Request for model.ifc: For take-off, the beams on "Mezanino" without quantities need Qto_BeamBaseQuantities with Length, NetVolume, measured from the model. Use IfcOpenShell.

First a look at what the model holds.

```python
import ifcopenshell
import ifcopenshell.util.element
import ifcopenshell.util.unit

model = ifcopenshell.open("model.ifc")
print(model.schema)
for unit_type in ("LENGTHUNIT", "AREAUNIT", "VOLUMEUNIT"):
    print(unit_type, ifcopenshell.util.unit.calculate_unit_scale(model, unit_type))
storey = next(s for s in model.by_type("IfcBuildingStorey") if s.Name == "Mezanino")
beams = [e for e in ifcopenshell.util.element.get_decomposition(storey) if e.is_a("IfcBeam")]
for e in sorted(beams, key=lambda e: e.id()):
    print(e.id(), e.is_a(), e.Name, list(ifcopenshell.util.element.get_psets(e, qtos_only=True)), sep=" | ")
```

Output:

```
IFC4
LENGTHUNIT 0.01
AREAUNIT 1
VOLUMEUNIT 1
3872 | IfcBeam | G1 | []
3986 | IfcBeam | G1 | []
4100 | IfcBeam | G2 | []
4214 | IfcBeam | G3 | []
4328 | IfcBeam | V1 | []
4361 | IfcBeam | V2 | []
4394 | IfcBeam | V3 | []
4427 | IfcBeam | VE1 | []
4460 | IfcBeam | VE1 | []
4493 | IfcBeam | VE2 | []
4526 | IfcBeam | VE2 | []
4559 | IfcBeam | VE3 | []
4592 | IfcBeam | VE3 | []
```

```python
import ifcopenshell
import ifcopenshell.api.pset
import ifcopenshell.geom
import ifcopenshell.util.element
import ifcopenshell.util.shape
import ifcopenshell.util.unit

model = ifcopenshell.open("model.ifc")
unit_scale = ifcopenshell.util.unit.calculate_unit_scale(model)
volume_scale = ifcopenshell.util.unit.calculate_unit_scale(model, "VOLUMEUNIT")
settings = ifcopenshell.geom.settings()

storey = next(s for s in model.by_type("IfcBuildingStorey") if s.Name == "Mezanino")
beams = [e for e in ifcopenshell.util.element.get_decomposition(storey) if e.is_a("IfcBeam")]

for e in sorted(beams, key=lambda e: e.id()):
    if ifcopenshell.util.element.get_psets(e, qtos_only=True, should_inherit=False):
        continue
    # Geometry comes back in metres, in the element's own axes.
    shape = ifcopenshell.geom.create_shape(settings, e)
    values = {
        "Length": ifcopenshell.util.shape.get_max_xyz(shape.geometry) / unit_scale,
        "NetVolume": ifcopenshell.util.shape.get_volume(shape.geometry) / volume_scale,
    }
    qto = ifcopenshell.api.pset.add_qto(model, product=e, name="Qto_BeamBaseQuantities")
    ifcopenshell.api.pset.edit_qto(model, qto=qto, properties=values)
    print(e.id(), {k: round(v, 3) for k, v in values.items()})

model.write("model_updated.ifc")
```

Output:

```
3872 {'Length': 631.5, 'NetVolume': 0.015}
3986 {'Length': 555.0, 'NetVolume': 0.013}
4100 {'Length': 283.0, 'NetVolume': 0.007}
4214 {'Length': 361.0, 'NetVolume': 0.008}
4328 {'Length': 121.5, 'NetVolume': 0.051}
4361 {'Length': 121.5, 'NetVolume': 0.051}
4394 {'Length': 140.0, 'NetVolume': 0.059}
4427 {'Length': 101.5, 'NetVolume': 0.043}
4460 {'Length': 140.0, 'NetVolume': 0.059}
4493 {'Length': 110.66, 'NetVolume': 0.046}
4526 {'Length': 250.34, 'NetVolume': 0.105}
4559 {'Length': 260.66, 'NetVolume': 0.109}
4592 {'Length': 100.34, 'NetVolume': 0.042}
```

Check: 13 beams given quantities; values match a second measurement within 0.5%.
